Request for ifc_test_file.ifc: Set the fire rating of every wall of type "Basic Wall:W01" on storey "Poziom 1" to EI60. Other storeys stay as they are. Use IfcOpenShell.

First a look at what the model holds.

```python
import ifcopenshell
import ifcopenshell.util.element

model = ifcopenshell.open("ifc_test_file.ifc")
print(model.schema)
storey = next(s for s in model.by_type("IfcBuildingStorey") if s.Name == "Poziom 1")
walls = [e for e in ifcopenshell.util.element.get_decomposition(storey) if e.is_a("IfcWall")]
seen = {}
for e in walls:
    element_type = ifcopenshell.util.element.get_type(e)
    key = (element_type.Name if element_type != e and element_type else None, ifcopenshell.util.element.get_pset(e, "Pset_WallCommon", "FireRating"))
    seen[key] = seen.get(key, 0) + 1
for (name, value), count in sorted(seen.items(), key=str):
    print(count, "x", name, "|", value)
```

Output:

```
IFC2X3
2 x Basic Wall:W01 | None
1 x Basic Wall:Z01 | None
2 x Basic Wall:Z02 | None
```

```python
import ifcopenshell
import ifcopenshell.api.pset
import ifcopenshell.util.element

model = ifcopenshell.open("ifc_test_file.ifc")

storey = next(s for s in model.by_type("IfcBuildingStorey") if s.Name == "Poziom 1")
walls = [e for e in ifcopenshell.util.element.get_decomposition(storey) if e.is_a("IfcWall")]

count = 0
for e in walls:
    element_type = ifcopenshell.util.element.get_type(e)
    if element_type in (None, e) or element_type.Name != "Basic Wall:W01":
        continue
    # add_pset returns the element's existing set when there is one.
    pset = ifcopenshell.api.pset.add_pset(model, product=e, name="Pset_WallCommon")
    ifcopenshell.api.pset.edit_pset(model, pset=pset, properties={"FireRating": "EI60"})
    count += 1

print(count, "walls updated")

model.write("ifc_test_file_v2.ifc")
```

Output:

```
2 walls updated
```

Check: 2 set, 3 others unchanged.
